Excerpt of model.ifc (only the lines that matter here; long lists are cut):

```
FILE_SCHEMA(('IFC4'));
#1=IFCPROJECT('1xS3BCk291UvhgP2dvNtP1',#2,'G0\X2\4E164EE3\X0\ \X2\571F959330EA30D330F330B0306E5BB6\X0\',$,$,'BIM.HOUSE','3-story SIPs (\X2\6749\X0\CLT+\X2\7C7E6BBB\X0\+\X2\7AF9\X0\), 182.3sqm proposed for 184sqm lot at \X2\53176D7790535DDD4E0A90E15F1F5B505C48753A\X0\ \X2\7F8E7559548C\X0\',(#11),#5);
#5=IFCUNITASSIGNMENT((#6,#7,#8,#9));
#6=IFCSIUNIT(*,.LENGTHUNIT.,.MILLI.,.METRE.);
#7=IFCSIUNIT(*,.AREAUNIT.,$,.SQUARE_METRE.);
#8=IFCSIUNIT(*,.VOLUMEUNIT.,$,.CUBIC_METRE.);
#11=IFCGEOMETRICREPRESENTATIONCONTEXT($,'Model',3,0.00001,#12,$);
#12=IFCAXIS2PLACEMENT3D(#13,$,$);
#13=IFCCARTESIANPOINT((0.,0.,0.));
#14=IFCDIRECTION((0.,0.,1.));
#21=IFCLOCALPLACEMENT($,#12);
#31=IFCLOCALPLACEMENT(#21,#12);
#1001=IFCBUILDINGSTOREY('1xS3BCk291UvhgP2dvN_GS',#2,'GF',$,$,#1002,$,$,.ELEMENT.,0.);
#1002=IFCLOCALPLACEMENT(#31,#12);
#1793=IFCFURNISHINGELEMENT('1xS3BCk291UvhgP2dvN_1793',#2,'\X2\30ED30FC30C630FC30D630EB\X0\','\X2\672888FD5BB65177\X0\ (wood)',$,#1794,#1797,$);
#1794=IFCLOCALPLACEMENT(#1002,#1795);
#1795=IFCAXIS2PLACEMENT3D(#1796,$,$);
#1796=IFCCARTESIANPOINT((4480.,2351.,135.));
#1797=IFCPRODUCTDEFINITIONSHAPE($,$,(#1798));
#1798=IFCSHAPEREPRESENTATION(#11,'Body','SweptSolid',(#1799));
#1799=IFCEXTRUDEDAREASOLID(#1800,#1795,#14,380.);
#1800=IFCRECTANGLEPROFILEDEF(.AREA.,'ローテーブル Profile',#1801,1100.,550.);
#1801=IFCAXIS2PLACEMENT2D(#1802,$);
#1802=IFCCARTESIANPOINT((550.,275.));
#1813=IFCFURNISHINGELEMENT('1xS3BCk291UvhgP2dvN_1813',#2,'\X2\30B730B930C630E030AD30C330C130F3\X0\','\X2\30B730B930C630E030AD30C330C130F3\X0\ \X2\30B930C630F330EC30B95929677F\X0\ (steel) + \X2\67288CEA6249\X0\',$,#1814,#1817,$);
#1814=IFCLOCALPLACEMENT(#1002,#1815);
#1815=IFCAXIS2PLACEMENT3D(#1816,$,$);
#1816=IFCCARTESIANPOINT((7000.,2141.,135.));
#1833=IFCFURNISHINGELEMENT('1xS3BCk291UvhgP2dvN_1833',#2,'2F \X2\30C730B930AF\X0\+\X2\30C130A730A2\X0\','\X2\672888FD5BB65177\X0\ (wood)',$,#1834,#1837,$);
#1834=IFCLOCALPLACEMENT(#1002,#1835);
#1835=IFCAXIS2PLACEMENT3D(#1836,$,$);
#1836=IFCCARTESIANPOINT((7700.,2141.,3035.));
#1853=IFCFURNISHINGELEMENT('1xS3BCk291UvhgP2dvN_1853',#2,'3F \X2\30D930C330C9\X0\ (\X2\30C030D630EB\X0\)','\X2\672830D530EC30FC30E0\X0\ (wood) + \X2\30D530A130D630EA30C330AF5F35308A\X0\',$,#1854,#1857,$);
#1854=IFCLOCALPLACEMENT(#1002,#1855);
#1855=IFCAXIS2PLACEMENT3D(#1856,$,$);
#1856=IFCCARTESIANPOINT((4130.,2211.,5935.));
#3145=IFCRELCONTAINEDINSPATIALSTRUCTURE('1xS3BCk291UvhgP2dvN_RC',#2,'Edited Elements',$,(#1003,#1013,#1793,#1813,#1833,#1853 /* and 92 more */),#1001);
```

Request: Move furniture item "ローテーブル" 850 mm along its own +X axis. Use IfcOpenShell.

```python
import ifcopenshell
import ifcopenshell.api.geometry
import ifcopenshell.util.placement
import ifcopenshell.util.unit

model = ifcopenshell.open("model.ifc")
unit_scale = ifcopenshell.util.unit.calculate_unit_scale(model)

item = model.by_guid("1xS3BCk291UvhgP2dvN_1793")
matrix = ifcopenshell.util.placement.get_local_placement(item.ObjectPlacement)
matrix[:3, 3] += matrix[:3, 0] * 0.85 / unit_scale
ifcopenshell.api.geometry.edit_object_placement(model, product=item, matrix=matrix, is_si=False)

print(ifcopenshell.util.placement.get_local_placement(item.ObjectPlacement).round(3) + 0.0)

model.write("model_v2.ifc")
```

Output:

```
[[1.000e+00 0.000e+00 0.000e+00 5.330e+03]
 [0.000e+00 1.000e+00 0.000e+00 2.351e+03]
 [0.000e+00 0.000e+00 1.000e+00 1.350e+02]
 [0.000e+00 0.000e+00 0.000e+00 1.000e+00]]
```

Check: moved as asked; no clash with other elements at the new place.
